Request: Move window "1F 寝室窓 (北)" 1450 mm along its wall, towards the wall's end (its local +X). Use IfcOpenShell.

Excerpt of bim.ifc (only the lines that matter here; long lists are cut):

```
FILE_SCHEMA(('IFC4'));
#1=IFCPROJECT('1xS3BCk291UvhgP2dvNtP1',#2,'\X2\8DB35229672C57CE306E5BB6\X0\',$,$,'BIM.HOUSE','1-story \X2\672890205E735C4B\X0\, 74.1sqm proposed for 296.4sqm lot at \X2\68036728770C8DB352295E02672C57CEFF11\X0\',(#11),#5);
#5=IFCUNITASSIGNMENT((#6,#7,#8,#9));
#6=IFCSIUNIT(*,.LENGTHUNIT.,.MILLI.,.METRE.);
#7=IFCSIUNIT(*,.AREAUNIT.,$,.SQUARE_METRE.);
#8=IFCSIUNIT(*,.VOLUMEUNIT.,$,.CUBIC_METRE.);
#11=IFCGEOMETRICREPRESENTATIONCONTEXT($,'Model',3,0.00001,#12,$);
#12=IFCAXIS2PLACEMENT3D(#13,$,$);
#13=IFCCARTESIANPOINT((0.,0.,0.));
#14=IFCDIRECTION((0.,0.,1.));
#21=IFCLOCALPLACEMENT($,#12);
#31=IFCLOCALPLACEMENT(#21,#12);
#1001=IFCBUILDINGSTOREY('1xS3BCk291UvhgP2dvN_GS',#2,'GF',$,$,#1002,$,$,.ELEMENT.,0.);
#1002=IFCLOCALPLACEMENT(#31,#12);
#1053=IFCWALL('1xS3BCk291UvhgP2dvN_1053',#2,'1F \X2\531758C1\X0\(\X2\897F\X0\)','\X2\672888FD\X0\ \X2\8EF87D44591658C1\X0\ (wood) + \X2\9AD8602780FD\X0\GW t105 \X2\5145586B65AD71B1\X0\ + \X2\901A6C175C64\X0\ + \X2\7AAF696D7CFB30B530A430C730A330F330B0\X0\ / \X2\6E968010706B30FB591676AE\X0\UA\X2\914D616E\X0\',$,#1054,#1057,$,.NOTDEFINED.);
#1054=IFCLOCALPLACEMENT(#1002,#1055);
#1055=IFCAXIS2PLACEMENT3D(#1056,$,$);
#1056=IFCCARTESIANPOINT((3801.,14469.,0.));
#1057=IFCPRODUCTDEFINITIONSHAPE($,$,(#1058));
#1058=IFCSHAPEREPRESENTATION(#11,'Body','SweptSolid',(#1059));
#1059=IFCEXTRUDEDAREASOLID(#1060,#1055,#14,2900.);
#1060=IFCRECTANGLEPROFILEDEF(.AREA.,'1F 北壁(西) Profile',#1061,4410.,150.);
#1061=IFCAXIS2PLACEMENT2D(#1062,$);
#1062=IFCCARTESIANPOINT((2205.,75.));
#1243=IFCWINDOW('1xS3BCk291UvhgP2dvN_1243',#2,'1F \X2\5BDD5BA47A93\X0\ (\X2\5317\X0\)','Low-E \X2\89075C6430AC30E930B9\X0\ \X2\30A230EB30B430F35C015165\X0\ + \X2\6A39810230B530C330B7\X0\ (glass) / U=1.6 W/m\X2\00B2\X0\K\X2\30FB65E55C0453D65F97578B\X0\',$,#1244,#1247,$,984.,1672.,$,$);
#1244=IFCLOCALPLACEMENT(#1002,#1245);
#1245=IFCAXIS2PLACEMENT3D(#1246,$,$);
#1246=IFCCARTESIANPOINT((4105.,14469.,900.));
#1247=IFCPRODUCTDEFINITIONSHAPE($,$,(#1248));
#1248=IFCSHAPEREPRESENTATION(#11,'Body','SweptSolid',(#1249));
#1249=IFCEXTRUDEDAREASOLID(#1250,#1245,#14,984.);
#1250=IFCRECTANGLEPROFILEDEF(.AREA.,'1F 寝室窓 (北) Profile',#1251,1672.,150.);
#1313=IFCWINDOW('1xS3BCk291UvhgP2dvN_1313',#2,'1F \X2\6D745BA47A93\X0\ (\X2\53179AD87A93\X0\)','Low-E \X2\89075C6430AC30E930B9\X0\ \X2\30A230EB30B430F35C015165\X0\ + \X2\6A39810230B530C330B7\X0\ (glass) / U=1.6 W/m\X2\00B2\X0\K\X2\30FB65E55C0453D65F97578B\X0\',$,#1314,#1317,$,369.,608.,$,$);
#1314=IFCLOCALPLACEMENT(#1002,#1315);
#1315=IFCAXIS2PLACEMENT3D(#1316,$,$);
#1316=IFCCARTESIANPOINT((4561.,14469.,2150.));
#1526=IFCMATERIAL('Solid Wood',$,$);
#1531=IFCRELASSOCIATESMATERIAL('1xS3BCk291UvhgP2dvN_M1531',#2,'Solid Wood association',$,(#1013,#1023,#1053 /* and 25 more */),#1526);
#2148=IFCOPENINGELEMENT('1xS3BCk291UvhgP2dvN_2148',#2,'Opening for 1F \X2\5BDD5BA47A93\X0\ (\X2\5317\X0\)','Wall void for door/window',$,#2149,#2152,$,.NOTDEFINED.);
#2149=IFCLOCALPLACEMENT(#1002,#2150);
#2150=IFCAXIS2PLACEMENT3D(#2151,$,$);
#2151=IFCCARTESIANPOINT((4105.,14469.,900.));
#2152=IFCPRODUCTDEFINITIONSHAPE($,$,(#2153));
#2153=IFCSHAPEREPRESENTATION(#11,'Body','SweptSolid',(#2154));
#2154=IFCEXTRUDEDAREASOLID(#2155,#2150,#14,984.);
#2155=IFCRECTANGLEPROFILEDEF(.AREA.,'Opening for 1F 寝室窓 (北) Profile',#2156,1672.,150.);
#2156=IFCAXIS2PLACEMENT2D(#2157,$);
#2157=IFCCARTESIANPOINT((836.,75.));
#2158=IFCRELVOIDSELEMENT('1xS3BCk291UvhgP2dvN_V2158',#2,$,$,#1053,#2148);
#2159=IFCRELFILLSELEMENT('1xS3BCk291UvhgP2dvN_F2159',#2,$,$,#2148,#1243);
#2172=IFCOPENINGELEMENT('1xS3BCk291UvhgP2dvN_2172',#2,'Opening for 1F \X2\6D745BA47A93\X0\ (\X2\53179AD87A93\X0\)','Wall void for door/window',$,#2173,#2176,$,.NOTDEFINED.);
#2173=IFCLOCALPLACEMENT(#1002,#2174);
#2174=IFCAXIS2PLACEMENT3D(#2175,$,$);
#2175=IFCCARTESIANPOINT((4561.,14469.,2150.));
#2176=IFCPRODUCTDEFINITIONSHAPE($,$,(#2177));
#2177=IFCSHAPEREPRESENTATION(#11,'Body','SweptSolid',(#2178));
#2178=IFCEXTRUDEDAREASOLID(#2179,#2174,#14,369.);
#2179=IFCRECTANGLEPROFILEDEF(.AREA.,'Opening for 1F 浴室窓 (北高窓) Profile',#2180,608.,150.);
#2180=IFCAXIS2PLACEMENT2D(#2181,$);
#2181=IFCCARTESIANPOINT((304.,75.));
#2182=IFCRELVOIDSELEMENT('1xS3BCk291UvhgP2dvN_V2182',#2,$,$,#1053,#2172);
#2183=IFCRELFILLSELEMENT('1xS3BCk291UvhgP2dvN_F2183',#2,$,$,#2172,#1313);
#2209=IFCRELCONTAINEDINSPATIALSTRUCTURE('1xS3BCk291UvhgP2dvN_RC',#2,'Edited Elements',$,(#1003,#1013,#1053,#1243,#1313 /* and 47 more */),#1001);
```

```python
import ifcopenshell
import ifcopenshell.api.geometry
import ifcopenshell.util.placement

model = ifcopenshell.open("bim.ifc")

window = model.by_guid("1xS3BCk291UvhgP2dvN_1243")
opening = window.FillsVoids[0].RelatingOpeningElement
wall = opening.VoidsElements[0].RelatingBuildingElement

wall_matrix = ifcopenshell.util.placement.get_local_placement(wall.ObjectPlacement)
shift = wall_matrix[:3, 0] * 1450.0
before = ifcopenshell.util.placement.get_local_placement(window.ObjectPlacement)[:3, 3].copy()

# The window is not placed relative to its opening, so move both.
for product in (opening, window):
    matrix = ifcopenshell.util.placement.get_local_placement(product.ObjectPlacement)
    matrix[:3, 3] += shift
    ifcopenshell.api.geometry.edit_object_placement(model, product=product, matrix=matrix, is_si=False)

after = ifcopenshell.util.placement.get_local_placement(window.ObjectPlacement)[:3, 3]
print("window moved by", (after - before).round(3) + 0.0)

model.write("bim_rev.ifc")
```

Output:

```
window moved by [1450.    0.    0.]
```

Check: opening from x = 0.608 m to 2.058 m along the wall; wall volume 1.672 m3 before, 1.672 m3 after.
